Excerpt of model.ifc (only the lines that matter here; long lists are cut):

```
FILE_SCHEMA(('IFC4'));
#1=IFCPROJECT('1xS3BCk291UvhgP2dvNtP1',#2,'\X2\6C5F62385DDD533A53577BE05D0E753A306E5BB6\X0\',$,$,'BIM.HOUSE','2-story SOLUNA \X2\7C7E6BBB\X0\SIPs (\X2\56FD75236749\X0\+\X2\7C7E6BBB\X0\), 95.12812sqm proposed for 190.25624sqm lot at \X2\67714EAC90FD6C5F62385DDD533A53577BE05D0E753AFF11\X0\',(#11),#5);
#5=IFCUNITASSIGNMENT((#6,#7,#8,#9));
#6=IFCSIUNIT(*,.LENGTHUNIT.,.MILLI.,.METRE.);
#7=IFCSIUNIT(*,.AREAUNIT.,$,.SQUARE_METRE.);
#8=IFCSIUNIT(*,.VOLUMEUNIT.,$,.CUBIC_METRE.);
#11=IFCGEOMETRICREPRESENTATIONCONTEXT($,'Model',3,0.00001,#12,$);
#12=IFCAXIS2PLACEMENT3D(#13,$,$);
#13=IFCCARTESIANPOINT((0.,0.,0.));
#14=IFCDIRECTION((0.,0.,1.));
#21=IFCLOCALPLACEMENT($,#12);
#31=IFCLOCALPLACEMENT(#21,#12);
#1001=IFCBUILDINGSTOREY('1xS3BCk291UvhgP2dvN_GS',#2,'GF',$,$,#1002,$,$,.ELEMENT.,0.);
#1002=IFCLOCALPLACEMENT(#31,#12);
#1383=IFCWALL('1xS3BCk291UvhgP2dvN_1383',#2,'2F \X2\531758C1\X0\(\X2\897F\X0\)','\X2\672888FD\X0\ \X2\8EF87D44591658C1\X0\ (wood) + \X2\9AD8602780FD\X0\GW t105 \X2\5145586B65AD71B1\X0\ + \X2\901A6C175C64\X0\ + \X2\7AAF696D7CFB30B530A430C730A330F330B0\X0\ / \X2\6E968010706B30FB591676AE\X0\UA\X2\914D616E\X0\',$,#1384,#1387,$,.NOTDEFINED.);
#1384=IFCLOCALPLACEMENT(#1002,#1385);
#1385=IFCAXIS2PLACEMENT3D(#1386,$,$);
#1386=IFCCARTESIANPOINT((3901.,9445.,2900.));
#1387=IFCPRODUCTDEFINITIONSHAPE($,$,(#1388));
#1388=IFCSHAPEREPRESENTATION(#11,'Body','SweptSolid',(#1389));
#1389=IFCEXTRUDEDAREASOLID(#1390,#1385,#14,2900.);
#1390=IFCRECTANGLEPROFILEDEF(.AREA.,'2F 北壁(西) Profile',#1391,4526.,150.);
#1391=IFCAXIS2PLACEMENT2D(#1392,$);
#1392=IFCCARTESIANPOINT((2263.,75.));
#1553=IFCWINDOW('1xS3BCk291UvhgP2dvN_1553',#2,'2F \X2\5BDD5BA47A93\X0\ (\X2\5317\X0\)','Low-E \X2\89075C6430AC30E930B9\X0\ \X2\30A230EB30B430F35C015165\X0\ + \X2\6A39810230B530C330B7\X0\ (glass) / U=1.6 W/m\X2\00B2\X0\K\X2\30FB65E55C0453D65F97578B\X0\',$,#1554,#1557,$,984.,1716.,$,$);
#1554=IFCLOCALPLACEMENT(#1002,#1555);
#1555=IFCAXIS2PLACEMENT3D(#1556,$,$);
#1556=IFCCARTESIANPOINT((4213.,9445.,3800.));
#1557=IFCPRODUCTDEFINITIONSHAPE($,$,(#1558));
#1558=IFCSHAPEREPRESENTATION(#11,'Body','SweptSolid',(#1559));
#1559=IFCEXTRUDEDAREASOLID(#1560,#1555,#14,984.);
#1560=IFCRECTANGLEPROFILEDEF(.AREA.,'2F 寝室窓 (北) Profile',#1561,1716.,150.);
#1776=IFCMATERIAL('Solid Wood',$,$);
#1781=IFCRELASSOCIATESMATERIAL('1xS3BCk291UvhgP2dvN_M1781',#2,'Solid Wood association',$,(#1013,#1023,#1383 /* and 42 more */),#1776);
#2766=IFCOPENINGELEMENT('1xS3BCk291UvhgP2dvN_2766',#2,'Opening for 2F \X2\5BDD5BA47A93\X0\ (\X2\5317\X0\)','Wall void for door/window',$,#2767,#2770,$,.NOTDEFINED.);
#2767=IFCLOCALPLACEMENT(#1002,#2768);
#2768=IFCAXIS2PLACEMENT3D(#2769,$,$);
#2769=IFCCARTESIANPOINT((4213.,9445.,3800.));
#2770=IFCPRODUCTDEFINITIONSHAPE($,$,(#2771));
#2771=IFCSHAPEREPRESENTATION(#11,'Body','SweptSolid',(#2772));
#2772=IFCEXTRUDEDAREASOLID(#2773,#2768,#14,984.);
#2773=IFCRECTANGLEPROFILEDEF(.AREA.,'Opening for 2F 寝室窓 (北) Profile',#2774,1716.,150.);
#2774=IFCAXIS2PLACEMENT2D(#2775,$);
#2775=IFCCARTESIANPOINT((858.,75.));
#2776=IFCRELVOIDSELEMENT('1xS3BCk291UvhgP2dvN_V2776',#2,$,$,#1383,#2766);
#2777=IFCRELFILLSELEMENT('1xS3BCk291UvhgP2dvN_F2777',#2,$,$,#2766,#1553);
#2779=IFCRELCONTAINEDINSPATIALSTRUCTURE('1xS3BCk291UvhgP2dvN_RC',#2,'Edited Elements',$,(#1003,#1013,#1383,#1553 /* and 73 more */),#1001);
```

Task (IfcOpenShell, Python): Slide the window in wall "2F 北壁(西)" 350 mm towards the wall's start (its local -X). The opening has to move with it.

```python
import ifcopenshell
import ifcopenshell.api.geometry
import ifcopenshell.util.placement
import ifcopenshell.util.unit

model = ifcopenshell.open("model.ifc")
unit_scale = ifcopenshell.util.unit.calculate_unit_scale(model)

window = model.by_guid("1xS3BCk291UvhgP2dvN_1553")
opening = window.FillsVoids[0].RelatingOpeningElement
wall = opening.VoidsElements[0].RelatingBuildingElement

wall_matrix = ifcopenshell.util.placement.get_local_placement(wall.ObjectPlacement)
shift = wall_matrix[:3, 0] * -0.35 / unit_scale
before = ifcopenshell.util.placement.get_local_placement(window.ObjectPlacement)[:3, 3].copy()

# The window is not placed relative to its opening, so move both.
for product in (opening, window):
    matrix = ifcopenshell.util.placement.get_local_placement(product.ObjectPlacement)
    matrix[:3, 3] += shift
    ifcopenshell.api.geometry.edit_object_placement(model, product=product, matrix=matrix, is_si=False)

after = ifcopenshell.util.placement.get_local_placement(window.ObjectPlacement)[:3, 3]
print("window moved by", (after - before).round(3) + 0.0)

model.write("model_updated.ifc")
```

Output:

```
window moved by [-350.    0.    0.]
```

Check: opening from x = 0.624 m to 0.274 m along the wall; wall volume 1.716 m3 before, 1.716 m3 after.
